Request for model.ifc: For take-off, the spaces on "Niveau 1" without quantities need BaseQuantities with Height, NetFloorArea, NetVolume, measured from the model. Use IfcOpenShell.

First a look at what the model holds.

```python
import ifcopenshell
import ifcopenshell.util.element
import ifcopenshell.util.unit

model = ifcopenshell.open("model.ifc")
print(model.schema)
for unit_type in ("LENGTHUNIT", "AREAUNIT", "VOLUMEUNIT"):
    print(unit_type, ifcopenshell.util.unit.calculate_unit_scale(model, unit_type))
storey = next(s for s in model.by_type("IfcBuildingStorey") if s.Name == "Niveau 1")
spaces = [e for e in ifcopenshell.util.element.get_decomposition(storey) if e.is_a("IfcSpace")]
for e in sorted(spaces, key=lambda e: e.id()):
    print(e.id(), e.is_a(), e.Name, list(ifcopenshell.util.element.get_psets(e, qtos_only=True)), sep=" | ")
```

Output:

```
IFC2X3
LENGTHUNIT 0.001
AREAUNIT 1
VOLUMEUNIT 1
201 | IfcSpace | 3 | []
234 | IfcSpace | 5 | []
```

```python
import ifcopenshell
import ifcopenshell.api.pset
import ifcopenshell.geom
import ifcopenshell.util.element
import ifcopenshell.util.shape
import ifcopenshell.util.unit

model = ifcopenshell.open("model.ifc")
unit_scale = ifcopenshell.util.unit.calculate_unit_scale(model)
area_scale = ifcopenshell.util.unit.calculate_unit_scale(model, "AREAUNIT")
volume_scale = ifcopenshell.util.unit.calculate_unit_scale(model, "VOLUMEUNIT")
settings = ifcopenshell.geom.settings()

storey = next(s for s in model.by_type("IfcBuildingStorey") if s.Name == "Niveau 1")
spaces = [e for e in ifcopenshell.util.element.get_decomposition(storey) if e.is_a("IfcSpace")]

for e in sorted(spaces, key=lambda e: e.id()):
    if ifcopenshell.util.element.get_psets(e, qtos_only=True, should_inherit=False):
        continue
    # Geometry comes back in metres, in the element's own axes.
    shape = ifcopenshell.geom.create_shape(settings, e)
    values = {
        "Height": ifcopenshell.util.shape.get_z(shape.geometry) / unit_scale,
        "NetFloorArea": ifcopenshell.util.shape.get_footprint_area(shape.geometry) / area_scale,
        "NetVolume": ifcopenshell.util.shape.get_volume(shape.geometry) / volume_scale,
    }
    qto = ifcopenshell.api.pset.add_qto(model, product=e, name="BaseQuantities")
    ifcopenshell.api.pset.edit_qto(model, qto=qto, properties=values)
    print(e.id(), {k: round(v, 3) for k, v in values.items()})

model.write("model_edited.ifc")
```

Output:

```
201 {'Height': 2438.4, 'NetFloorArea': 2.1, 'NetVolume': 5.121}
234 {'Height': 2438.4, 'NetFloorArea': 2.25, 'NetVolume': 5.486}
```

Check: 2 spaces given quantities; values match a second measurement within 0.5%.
